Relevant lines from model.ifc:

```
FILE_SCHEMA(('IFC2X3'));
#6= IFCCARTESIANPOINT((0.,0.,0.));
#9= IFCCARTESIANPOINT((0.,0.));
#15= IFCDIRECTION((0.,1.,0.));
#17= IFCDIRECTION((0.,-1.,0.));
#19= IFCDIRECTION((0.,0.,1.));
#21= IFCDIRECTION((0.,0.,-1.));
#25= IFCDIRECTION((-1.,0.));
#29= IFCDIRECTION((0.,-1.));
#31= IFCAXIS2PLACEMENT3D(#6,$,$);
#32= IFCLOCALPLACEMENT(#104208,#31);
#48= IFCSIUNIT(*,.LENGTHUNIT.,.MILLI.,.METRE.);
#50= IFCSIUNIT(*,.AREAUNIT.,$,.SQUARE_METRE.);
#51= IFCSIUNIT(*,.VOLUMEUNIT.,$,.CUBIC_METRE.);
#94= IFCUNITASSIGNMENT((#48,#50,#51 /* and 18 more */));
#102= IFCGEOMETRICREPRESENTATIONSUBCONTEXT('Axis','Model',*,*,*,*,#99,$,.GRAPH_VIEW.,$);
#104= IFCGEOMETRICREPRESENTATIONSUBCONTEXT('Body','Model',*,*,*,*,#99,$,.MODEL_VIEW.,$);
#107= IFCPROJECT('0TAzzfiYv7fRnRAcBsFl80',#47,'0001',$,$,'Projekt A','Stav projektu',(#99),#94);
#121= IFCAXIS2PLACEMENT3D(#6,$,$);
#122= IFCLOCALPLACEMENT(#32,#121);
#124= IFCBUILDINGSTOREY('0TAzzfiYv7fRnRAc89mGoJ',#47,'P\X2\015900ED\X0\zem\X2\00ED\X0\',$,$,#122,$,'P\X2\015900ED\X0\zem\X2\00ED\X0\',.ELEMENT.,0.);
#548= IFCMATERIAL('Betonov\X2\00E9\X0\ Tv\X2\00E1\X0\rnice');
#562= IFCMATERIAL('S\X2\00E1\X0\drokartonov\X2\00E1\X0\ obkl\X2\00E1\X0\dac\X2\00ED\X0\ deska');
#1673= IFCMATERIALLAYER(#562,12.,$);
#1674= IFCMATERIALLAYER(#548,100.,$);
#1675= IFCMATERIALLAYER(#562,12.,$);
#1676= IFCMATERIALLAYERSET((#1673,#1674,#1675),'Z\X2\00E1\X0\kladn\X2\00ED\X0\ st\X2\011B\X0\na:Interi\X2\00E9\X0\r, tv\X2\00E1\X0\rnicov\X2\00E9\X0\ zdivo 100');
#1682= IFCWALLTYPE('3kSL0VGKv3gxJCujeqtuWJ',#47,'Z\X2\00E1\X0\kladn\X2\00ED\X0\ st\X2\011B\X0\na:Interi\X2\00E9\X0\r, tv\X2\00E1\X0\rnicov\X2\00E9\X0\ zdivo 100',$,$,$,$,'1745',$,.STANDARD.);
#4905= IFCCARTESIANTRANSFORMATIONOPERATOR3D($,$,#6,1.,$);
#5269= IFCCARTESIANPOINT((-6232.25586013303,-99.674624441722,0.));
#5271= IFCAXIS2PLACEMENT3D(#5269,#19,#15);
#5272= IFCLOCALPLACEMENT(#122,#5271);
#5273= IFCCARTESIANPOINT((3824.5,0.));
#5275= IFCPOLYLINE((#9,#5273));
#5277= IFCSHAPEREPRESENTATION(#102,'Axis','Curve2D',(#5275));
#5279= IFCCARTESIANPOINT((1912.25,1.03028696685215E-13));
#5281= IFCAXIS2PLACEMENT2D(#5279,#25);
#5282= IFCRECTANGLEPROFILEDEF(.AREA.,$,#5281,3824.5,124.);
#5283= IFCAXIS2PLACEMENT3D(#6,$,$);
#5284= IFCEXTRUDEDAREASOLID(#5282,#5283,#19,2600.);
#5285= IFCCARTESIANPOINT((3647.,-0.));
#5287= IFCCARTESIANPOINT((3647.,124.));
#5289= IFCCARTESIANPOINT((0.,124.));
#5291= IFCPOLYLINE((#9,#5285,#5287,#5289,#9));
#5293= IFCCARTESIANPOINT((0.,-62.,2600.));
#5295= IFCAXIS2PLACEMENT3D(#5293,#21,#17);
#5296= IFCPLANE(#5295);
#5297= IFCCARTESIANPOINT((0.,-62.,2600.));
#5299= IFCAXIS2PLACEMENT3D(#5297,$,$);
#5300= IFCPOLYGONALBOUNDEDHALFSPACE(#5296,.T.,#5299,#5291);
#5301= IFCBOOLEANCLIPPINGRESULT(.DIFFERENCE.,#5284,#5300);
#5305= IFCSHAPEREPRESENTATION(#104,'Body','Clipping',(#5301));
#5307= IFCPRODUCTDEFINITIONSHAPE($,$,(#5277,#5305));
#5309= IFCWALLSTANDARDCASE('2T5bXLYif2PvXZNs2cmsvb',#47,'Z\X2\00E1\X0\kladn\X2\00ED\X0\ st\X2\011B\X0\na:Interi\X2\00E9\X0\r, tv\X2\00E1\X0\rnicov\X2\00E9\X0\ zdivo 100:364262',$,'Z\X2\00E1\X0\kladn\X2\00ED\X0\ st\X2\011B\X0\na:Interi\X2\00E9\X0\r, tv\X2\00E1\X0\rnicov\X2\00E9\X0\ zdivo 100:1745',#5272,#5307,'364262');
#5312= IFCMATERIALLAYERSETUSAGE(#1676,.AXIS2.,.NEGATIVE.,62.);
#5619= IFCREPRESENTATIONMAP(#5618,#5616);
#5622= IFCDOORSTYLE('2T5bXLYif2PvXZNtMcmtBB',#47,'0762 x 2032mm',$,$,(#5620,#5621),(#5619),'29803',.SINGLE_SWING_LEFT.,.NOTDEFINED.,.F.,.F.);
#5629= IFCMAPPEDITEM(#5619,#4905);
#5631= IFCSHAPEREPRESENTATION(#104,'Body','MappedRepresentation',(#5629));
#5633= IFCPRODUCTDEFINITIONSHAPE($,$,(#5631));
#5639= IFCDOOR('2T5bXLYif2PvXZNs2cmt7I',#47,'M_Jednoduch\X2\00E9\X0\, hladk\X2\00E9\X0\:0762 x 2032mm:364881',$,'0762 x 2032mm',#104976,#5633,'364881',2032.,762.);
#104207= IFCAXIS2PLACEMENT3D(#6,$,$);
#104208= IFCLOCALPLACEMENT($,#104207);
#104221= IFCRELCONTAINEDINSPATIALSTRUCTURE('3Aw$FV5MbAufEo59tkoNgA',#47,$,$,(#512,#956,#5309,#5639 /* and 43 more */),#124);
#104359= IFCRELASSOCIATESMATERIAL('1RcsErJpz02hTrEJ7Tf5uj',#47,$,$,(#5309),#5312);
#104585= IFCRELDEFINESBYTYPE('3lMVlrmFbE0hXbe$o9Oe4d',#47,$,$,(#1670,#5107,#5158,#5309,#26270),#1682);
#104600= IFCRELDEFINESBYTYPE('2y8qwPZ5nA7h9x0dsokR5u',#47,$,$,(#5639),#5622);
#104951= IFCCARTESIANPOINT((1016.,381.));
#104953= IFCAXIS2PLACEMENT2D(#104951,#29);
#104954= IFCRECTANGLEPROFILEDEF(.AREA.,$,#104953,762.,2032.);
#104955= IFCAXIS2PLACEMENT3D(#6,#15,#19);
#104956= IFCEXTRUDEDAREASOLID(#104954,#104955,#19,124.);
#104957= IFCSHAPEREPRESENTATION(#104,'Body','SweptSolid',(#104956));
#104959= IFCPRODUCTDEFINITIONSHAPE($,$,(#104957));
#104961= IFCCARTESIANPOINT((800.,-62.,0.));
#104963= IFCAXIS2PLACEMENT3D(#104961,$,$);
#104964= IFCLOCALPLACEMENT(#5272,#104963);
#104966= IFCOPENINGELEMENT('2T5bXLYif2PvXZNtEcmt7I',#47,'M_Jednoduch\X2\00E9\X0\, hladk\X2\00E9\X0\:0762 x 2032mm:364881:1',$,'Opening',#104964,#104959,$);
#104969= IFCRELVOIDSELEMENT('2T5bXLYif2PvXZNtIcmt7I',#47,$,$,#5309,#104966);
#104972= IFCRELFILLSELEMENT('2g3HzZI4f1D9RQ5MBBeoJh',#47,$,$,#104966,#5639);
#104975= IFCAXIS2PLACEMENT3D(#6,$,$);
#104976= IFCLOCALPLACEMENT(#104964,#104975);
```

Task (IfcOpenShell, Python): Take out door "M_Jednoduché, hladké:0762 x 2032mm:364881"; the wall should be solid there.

```python
import ifcopenshell
import ifcopenshell.api.feature
import ifcopenshell.api.root
import ifcopenshell.geom
import ifcopenshell.util.shape

model = ifcopenshell.open("model.ifc")
settings = ifcopenshell.geom.settings()


def volume(element):
    """Net volume in cubic metres, openings subtracted."""
    shape = ifcopenshell.geom.create_shape(settings, element)
    return ifcopenshell.util.shape.get_volume(shape.geometry)


door = model.by_id(5639)
opening = door.FillsVoids[0].RelatingOpeningElement
wall = opening.VoidsElements[0].RelatingBuildingElement
before = volume(wall)

ifcopenshell.api.root.remove_product(model, product=door)
ifcopenshell.api.feature.remove_feature(model, feature=opening)

after = volume(wall)

print(f"wall volume {before:.3f} -> {after:.3f} m3")

model.write("model_v2.ifc")
```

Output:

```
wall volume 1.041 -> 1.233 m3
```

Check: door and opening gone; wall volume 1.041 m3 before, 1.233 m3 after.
